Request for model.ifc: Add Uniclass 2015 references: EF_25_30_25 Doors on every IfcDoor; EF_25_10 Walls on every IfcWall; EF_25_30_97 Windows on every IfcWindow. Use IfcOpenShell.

First a look at what the model holds.

```python
import ifcopenshell

model = ifcopenshell.open("model.ifc")
print(model.schema)
print("classifications:", [c.Name for c in model.by_type("IfcClassification")])
for ifc_class in ("IfcDoor", "IfcRoof", "IfcStair", "IfcWall", "IfcWindow"):
    print(ifc_class, len(model.by_type(ifc_class)))
```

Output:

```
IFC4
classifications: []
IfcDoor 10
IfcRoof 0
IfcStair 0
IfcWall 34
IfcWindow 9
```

```python
import ifcopenshell
import ifcopenshell.api.classification

model = ifcopenshell.open("model.ifc")

system = ifcopenshell.api.classification.add_classification(model, classification="Uniclass 2015")

codes = {
    "IfcDoor": ("EF_25_30_25", "Doors"),
    "IfcWall": ("EF_25_10", "Walls"),
    "IfcWindow": ("EF_25_30_97", "Windows"),
}
for ifc_class, (code, name) in codes.items():
    products = model.by_type(ifc_class)
    ifcopenshell.api.classification.add_reference(
        model, products=products, classification=system, identification=code, name=name
    )
    print(code, len(products))

model.write("model_edited.ifc")
```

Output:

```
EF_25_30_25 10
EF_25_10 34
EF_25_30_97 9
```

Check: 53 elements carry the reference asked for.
